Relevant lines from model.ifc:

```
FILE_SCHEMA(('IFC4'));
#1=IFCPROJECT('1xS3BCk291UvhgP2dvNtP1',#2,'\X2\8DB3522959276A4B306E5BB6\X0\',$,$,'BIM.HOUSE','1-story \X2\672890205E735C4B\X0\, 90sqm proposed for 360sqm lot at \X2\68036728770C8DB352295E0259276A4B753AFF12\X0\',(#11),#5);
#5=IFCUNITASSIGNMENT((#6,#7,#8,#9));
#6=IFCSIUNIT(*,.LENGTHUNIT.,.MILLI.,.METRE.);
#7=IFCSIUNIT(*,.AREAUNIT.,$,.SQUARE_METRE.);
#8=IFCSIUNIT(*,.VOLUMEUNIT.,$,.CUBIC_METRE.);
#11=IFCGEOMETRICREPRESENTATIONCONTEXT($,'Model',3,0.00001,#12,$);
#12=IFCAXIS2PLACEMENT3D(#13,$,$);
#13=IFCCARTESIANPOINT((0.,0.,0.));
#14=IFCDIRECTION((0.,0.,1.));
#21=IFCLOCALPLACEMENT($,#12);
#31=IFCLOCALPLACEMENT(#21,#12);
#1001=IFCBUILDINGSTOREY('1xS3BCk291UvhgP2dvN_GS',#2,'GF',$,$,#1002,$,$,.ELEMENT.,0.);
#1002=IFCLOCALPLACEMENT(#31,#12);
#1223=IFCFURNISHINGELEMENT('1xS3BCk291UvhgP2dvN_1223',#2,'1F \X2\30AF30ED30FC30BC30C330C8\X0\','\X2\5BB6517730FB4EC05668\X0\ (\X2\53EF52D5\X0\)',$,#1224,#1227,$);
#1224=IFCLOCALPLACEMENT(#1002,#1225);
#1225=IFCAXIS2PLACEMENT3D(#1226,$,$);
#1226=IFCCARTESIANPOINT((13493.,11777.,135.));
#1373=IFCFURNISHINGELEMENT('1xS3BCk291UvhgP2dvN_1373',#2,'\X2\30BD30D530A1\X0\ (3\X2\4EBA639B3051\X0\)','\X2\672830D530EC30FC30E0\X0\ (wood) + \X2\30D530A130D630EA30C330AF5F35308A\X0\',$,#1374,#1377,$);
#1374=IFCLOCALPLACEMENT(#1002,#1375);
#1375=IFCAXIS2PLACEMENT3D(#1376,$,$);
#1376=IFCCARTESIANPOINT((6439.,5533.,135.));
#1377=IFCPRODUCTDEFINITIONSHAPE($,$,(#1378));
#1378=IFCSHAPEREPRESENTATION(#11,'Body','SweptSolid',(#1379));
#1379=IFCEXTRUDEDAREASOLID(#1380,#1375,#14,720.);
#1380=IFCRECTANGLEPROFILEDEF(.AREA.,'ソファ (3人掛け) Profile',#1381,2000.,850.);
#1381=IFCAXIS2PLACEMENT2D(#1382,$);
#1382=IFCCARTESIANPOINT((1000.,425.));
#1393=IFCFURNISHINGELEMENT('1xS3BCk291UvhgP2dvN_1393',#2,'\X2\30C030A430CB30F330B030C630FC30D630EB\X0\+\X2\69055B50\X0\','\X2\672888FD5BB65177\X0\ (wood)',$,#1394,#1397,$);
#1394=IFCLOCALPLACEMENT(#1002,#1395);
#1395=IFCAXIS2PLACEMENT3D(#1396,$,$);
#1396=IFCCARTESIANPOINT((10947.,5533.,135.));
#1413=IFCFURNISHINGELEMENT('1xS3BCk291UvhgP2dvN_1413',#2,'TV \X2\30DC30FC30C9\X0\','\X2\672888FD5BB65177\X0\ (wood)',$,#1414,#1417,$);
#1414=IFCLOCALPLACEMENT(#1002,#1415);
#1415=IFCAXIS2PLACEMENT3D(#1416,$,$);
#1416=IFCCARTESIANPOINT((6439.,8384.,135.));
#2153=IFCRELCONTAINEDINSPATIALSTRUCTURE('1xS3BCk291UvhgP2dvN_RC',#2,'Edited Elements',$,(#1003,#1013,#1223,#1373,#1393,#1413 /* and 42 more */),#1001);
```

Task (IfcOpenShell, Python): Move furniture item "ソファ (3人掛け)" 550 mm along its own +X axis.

```python
import ifcopenshell
import ifcopenshell.api.geometry
import ifcopenshell.util.placement
import ifcopenshell.util.unit

model = ifcopenshell.open("model.ifc")
unit_scale = ifcopenshell.util.unit.calculate_unit_scale(model)

item = model.by_guid("1xS3BCk291UvhgP2dvN_1373")
matrix = ifcopenshell.util.placement.get_local_placement(item.ObjectPlacement)
matrix[:3, 3] += matrix[:3, 0] * 0.55 / unit_scale
ifcopenshell.api.geometry.edit_object_placement(model, product=item, matrix=matrix, is_si=False)

print(ifcopenshell.util.placement.get_local_placement(item.ObjectPlacement).round(3) + 0.0)

model.write("model_edited.ifc")
```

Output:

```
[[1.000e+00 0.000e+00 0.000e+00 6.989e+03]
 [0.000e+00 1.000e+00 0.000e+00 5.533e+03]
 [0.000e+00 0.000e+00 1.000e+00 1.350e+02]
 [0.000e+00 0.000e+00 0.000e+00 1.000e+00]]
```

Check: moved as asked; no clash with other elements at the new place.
